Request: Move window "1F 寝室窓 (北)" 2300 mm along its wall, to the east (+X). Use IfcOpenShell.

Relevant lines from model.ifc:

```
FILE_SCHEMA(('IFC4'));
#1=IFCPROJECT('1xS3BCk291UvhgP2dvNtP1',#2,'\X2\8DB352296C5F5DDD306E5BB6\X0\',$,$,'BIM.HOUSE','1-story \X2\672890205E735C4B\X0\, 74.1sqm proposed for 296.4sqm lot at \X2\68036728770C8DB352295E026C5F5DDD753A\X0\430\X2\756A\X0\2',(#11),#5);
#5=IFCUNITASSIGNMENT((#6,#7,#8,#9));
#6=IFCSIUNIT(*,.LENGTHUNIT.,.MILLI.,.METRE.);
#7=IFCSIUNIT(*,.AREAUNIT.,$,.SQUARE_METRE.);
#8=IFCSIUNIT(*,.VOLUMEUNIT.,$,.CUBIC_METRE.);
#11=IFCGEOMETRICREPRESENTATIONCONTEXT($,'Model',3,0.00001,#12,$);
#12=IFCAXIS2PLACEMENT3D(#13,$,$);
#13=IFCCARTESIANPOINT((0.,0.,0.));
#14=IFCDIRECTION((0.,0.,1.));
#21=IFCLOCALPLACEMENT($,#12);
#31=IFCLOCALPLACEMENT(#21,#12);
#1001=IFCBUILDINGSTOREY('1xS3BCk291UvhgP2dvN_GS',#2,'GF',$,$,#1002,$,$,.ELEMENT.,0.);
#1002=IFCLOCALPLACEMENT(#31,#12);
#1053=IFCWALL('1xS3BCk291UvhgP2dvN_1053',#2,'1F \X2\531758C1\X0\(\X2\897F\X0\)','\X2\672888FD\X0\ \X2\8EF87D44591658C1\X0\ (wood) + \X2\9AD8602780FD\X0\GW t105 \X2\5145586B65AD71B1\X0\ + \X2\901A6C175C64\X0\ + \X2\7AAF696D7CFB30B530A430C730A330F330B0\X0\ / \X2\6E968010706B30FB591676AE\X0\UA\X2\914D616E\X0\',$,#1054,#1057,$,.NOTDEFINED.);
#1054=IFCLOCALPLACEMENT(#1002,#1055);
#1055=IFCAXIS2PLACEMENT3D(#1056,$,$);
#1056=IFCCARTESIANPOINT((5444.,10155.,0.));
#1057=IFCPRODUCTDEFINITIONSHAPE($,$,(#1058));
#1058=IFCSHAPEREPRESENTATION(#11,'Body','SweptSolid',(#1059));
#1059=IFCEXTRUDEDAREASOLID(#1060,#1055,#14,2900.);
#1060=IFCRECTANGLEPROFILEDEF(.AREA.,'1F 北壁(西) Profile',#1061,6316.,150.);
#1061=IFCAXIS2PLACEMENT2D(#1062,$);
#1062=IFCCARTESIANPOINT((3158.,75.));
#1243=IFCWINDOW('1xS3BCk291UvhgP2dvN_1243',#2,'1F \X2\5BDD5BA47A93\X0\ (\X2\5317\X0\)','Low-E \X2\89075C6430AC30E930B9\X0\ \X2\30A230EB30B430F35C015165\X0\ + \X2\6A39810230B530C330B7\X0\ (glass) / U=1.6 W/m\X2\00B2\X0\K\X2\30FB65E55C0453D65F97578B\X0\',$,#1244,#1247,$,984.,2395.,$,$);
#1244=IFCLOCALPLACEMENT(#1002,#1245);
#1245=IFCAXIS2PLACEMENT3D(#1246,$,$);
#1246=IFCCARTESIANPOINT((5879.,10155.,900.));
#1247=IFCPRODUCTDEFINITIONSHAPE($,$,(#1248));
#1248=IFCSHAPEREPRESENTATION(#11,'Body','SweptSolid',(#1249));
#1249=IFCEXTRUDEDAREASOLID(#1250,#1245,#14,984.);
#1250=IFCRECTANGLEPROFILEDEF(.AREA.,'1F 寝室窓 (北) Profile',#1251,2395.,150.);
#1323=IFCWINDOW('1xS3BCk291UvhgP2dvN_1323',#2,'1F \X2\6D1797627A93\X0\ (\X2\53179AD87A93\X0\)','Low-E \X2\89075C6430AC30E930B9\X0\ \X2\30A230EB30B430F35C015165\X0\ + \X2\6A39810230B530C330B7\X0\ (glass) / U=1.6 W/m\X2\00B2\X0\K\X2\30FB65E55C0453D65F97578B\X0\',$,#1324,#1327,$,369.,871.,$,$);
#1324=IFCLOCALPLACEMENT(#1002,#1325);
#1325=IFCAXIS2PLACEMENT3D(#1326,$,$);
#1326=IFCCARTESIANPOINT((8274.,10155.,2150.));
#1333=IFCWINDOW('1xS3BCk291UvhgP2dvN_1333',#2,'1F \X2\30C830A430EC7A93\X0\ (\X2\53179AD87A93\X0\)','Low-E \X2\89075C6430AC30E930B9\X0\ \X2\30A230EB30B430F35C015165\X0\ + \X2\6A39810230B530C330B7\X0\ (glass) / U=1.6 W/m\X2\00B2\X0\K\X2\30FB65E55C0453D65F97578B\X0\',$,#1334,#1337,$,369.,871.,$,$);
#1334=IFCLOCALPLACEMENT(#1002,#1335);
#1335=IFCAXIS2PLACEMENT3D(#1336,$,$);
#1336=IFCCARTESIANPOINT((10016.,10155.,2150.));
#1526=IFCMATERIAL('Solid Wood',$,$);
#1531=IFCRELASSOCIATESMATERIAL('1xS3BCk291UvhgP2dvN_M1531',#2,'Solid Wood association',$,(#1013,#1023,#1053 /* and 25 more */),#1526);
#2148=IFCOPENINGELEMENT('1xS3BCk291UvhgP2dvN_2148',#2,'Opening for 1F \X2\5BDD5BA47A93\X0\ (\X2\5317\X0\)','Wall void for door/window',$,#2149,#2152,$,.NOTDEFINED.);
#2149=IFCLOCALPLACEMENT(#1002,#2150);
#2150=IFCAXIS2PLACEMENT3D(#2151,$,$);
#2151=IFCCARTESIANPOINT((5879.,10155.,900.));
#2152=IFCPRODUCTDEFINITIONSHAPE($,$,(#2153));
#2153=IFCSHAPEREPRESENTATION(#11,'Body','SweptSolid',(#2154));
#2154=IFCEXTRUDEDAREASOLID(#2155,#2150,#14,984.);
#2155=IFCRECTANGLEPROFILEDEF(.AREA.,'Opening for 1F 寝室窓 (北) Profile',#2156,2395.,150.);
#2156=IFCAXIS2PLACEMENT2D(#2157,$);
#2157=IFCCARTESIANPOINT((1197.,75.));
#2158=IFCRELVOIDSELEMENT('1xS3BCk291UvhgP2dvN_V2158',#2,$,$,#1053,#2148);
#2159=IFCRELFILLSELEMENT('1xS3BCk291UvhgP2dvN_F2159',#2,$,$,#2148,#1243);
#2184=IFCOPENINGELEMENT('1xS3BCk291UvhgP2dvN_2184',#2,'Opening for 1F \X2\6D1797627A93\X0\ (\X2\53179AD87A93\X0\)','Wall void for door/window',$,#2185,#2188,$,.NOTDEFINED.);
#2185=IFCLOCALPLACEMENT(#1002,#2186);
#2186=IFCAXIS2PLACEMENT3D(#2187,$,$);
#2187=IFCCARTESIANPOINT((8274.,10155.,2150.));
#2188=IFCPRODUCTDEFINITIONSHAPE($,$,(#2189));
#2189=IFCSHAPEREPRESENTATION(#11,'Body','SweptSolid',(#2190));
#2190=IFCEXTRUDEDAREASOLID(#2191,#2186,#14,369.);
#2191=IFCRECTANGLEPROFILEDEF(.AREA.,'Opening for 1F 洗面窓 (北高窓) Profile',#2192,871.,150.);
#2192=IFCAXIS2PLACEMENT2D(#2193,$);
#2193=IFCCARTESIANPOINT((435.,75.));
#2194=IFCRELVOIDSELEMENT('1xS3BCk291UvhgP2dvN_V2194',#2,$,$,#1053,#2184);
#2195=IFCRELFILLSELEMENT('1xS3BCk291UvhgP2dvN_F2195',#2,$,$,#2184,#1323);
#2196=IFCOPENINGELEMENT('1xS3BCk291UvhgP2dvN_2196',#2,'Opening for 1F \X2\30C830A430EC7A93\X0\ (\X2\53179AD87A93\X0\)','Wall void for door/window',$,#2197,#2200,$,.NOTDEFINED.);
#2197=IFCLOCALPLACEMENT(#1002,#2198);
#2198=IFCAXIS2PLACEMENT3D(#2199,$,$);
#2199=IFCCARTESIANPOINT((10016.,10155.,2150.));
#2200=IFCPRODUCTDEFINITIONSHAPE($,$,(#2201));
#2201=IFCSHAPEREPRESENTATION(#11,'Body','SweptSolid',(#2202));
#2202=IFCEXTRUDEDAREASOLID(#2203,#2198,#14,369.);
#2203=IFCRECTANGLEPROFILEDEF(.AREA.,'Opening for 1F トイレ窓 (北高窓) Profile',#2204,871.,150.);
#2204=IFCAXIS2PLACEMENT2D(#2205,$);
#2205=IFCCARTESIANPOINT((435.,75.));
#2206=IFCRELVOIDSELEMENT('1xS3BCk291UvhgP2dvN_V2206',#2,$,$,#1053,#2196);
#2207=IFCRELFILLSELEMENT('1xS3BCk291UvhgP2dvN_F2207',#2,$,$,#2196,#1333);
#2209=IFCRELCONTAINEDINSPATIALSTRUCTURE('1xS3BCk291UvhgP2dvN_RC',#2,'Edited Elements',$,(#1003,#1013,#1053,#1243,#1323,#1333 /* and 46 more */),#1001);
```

```python
import ifcopenshell
import ifcopenshell.api.geometry
import ifcopenshell.util.placement
import ifcopenshell.util.unit

model = ifcopenshell.open("model.ifc")
unit_scale = ifcopenshell.util.unit.calculate_unit_scale(model)

window = model.by_guid("1xS3BCk291UvhgP2dvN_1243")
opening = window.FillsVoids[0].RelatingOpeningElement
wall = opening.VoidsElements[0].RelatingBuildingElement

wall_matrix = ifcopenshell.util.placement.get_local_placement(wall.ObjectPlacement)
shift = wall_matrix[:3, 0] * 2.3 / unit_scale
before = ifcopenshell.util.placement.get_local_placement(window.ObjectPlacement)[:3, 3].copy()

# The window is not placed relative to its opening, so move both.
for product in (opening, window):
    matrix = ifcopenshell.util.placement.get_local_placement(product.ObjectPlacement)
    matrix[:3, 3] += shift
    ifcopenshell.api.geometry.edit_object_placement(model, product=product, matrix=matrix, is_si=False)

after = ifcopenshell.util.placement.get_local_placement(window.ObjectPlacement)[:3, 3]
print("window moved by", (after - before).round(3) + 0.0)

model.write("model_edited.ifc")
```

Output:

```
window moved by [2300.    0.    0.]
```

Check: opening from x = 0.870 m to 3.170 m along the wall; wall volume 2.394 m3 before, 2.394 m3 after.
